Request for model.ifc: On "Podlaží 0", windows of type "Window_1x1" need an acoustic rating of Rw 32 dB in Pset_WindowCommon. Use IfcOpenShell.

First a look at what the model holds.

```python
import ifcopenshell
import ifcopenshell.util.element

model = ifcopenshell.open("model.ifc")
print(model.schema)
storey = next(s for s in model.by_type("IfcBuildingStorey") if s.Name == "Podlaží 0")
windows = [e for e in ifcopenshell.util.element.get_decomposition(storey) if e.is_a("IfcWindow")]
seen = {}
for e in windows:
    element_type = ifcopenshell.util.element.get_type(e)
    key = (element_type.Name if element_type != e and element_type else None, ifcopenshell.util.element.get_pset(e, "Pset_WindowCommon", "AcousticRating"))
    seen[key] = seen.get(key, 0) + 1
for (name, value), count in sorted(seen.items(), key=str):
    print(count, "x", name, "|", value)
```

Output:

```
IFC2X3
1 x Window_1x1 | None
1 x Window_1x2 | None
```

```python
import ifcopenshell
import ifcopenshell.api.pset
import ifcopenshell.util.element

model = ifcopenshell.open("model.ifc")

storey = next(s for s in model.by_type("IfcBuildingStorey") if s.Name == "Podlaží 0")
windows = [e for e in ifcopenshell.util.element.get_decomposition(storey) if e.is_a("IfcWindow")]

count = 0
for e in windows:
    element_type = ifcopenshell.util.element.get_type(e)
    if element_type in (None, e) or element_type.Name != "Window_1x1":
        continue
    # add_pset returns the element's existing set when there is one.
    pset = ifcopenshell.api.pset.add_pset(model, product=e, name="Pset_WindowCommon")
    ifcopenshell.api.pset.edit_pset(model, pset=pset, properties={"AcousticRating": "Rw 32 dB"})
    count += 1

print(count, "windows updated")

model.write("model_rev.ifc")
```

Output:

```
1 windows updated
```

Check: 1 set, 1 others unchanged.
